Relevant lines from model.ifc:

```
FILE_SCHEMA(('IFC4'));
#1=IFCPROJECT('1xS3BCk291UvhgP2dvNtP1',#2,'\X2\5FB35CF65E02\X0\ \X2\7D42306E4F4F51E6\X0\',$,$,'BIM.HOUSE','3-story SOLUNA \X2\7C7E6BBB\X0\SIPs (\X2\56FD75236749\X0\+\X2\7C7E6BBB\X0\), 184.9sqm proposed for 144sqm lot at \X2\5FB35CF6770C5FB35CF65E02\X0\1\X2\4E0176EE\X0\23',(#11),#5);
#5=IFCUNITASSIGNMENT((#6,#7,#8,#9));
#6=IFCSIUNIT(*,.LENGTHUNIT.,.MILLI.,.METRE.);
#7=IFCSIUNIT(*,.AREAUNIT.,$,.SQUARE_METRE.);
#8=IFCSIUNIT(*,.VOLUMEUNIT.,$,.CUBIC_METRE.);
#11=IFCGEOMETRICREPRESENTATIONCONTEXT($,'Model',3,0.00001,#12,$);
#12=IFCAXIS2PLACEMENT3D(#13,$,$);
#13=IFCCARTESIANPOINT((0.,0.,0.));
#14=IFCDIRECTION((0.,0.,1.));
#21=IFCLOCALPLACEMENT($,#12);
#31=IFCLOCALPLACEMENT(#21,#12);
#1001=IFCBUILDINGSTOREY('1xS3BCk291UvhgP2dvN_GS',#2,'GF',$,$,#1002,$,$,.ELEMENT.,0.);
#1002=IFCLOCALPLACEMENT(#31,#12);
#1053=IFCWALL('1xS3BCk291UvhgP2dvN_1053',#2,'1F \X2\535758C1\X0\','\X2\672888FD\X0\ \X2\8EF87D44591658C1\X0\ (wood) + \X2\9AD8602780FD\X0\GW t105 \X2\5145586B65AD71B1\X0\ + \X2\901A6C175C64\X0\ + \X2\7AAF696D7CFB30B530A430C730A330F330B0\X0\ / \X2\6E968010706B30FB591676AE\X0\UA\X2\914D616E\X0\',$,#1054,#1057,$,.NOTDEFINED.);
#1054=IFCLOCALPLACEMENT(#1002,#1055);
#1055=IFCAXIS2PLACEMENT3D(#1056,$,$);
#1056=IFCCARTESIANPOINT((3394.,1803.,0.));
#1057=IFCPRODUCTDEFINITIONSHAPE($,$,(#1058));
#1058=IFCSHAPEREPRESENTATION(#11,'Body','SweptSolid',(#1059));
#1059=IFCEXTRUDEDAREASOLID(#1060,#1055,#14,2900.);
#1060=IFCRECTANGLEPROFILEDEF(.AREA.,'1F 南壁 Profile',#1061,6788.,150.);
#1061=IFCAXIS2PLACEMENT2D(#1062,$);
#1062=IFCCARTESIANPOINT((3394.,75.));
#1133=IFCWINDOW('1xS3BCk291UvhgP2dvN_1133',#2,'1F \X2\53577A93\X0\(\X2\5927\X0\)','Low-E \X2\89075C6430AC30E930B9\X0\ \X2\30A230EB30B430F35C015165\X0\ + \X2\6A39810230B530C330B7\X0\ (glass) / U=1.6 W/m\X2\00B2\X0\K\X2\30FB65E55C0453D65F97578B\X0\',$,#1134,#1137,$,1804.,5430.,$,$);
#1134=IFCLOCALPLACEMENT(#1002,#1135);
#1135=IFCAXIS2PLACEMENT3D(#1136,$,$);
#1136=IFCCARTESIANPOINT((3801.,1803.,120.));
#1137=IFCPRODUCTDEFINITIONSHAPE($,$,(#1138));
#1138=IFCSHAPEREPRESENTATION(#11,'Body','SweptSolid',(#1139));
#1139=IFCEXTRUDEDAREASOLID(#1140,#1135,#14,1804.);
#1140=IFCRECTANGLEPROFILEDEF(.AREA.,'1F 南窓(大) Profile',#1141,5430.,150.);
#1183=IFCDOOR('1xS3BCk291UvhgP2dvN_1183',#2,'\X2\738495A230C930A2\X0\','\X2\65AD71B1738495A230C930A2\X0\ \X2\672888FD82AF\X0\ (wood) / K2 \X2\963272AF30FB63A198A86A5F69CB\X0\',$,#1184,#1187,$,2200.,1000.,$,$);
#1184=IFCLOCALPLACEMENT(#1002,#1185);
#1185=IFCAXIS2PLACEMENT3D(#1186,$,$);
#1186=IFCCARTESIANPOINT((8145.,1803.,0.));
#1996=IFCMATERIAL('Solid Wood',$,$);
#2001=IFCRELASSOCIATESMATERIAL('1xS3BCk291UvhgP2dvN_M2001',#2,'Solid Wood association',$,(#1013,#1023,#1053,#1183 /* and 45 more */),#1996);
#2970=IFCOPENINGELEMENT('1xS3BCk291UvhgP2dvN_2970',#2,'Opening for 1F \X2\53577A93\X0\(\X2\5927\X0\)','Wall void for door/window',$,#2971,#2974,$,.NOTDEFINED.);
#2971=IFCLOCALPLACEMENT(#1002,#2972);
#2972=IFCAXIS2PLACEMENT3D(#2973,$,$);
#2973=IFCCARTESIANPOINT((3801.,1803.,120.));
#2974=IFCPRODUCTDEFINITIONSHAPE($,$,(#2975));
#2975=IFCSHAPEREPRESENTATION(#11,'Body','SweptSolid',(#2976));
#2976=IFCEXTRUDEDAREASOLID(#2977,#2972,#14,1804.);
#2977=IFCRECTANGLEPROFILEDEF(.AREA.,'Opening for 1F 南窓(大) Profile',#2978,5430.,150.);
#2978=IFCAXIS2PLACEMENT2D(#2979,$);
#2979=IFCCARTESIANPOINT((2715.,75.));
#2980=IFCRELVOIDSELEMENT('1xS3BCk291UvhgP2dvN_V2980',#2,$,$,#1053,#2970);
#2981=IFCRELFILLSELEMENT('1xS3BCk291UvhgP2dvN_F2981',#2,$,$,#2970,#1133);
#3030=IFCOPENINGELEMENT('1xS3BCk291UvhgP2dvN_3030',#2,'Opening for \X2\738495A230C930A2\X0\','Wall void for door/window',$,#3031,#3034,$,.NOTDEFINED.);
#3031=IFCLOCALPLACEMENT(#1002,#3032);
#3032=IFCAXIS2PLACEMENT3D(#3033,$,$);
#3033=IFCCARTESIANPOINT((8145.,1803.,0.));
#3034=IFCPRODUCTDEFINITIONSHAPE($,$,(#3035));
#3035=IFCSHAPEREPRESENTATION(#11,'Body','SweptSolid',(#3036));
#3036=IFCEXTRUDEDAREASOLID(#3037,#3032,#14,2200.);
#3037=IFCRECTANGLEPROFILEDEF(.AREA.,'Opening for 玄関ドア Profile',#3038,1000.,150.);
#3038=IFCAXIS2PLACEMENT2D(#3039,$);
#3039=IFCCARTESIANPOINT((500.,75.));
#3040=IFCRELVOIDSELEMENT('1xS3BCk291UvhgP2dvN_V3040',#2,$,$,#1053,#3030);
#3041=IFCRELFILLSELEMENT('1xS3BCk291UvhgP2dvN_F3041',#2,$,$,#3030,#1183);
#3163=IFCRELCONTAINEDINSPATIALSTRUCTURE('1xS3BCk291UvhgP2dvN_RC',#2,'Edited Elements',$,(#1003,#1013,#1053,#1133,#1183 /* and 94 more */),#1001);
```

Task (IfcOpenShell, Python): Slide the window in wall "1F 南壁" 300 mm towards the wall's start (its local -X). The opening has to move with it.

```python
import ifcopenshell
import ifcopenshell.api.geometry
import ifcopenshell.util.placement

model = ifcopenshell.open("model.ifc")

window = model.by_guid("1xS3BCk291UvhgP2dvN_1133")
opening = window.FillsVoids[0].RelatingOpeningElement
wall = opening.VoidsElements[0].RelatingBuildingElement

wall_matrix = ifcopenshell.util.placement.get_local_placement(wall.ObjectPlacement)
shift = wall_matrix[:3, 0] * -300.0
before = ifcopenshell.util.placement.get_local_placement(window.ObjectPlacement)[:3, 3].copy()

# The window is not placed relative to its opening, so move both.
for product in (opening, window):
    matrix = ifcopenshell.util.placement.get_local_placement(product.ObjectPlacement)
    matrix[:3, 3] += shift
    ifcopenshell.api.geometry.edit_object_placement(model, product=product, matrix=matrix, is_si=False)

after = ifcopenshell.util.placement.get_local_placement(window.ObjectPlacement)[:3, 3]
print("window moved by", (after - before).round(3) + 0.0)

model.write("model-out.ifc")
```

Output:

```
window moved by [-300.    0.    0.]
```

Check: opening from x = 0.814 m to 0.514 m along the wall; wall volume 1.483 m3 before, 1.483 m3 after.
